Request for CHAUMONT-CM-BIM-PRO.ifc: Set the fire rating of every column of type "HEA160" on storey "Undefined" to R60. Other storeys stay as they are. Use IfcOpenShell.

First a look at what the model holds.

```python
import ifcopenshell
import ifcopenshell.util.element

model = ifcopenshell.open("CHAUMONT-CM-BIM-PRO.ifc")
print(model.schema)
storey = next(s for s in model.by_type("IfcBuildingStorey") if s.Name == "Undefined")
columns = [e for e in ifcopenshell.util.element.get_decomposition(storey) if e.is_a("IfcColumn")]
seen = {}
for e in columns:
    element_type = ifcopenshell.util.element.get_type(e)
    key = (element_type.Name if element_type != e and element_type else None, ifcopenshell.util.element.get_pset(e, "Pset_ColumnCommon", "FireRating"))
    seen[key] = seen.get(key, 0) + 1
for (name, value), count in sorted(seen.items(), key=str):
    print(count, "x", name, "|", value)
```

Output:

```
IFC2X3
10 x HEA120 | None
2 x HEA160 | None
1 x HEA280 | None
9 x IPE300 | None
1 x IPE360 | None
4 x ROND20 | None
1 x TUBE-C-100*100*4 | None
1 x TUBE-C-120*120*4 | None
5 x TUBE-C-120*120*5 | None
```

```python
import ifcopenshell
import ifcopenshell.api.pset
import ifcopenshell.util.element

model = ifcopenshell.open("CHAUMONT-CM-BIM-PRO.ifc")

storey = next(s for s in model.by_type("IfcBuildingStorey") if s.Name == "Undefined")
columns = [e for e in ifcopenshell.util.element.get_decomposition(storey) if e.is_a("IfcColumn")]

count = 0
for e in columns:
    element_type = ifcopenshell.util.element.get_type(e)
    if element_type in (None, e) or element_type.Name != "HEA160":
        continue
    found = ifcopenshell.util.element.get_pset(e, "Pset_ColumnCommon", should_inherit=False)
    if found:
        pset = model.by_id(found["id"])
        if len(ifcopenshell.util.element.get_elements_by_pset(pset)) > 1:
            pset = ifcopenshell.api.pset.unshare_pset(model, products=[e], pset=pset)[0]
    else:
        pset = ifcopenshell.api.pset.add_pset(model, product=e, name="Pset_ColumnCommon")
    ifcopenshell.api.pset.edit_pset(model, pset=pset, properties={"FireRating": "R60"})
    count += 1

print(count, "columns updated")

model.write("CHAUMONT-CM-BIM-PRO_rev.ifc")
```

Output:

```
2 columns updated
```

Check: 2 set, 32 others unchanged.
